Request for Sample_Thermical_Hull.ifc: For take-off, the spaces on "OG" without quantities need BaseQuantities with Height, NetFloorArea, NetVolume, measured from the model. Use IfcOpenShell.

First a look at what the model holds.

```python
import ifcopenshell
import ifcopenshell.util.element
import ifcopenshell.util.unit

model = ifcopenshell.open("Sample_Thermical_Hull.ifc")
print(model.schema)
for unit_type in ("LENGTHUNIT", "AREAUNIT", "VOLUMEUNIT"):
    print(unit_type, ifcopenshell.util.unit.calculate_unit_scale(model, unit_type))
storey = next(s for s in model.by_type("IfcBuildingStorey") if s.Name == "OG")
spaces = [e for e in ifcopenshell.util.element.get_decomposition(storey) if e.is_a("IfcSpace")]
for e in sorted(spaces, key=lambda e: e.id()):
    print(e.id(), e.is_a(), e.Name, list(ifcopenshell.util.element.get_psets(e, qtos_only=True)), sep=" | ")
```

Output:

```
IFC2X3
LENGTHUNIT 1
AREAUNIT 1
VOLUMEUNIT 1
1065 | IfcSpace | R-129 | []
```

```python
import ifcopenshell
import ifcopenshell.api.pset
import ifcopenshell.geom
import ifcopenshell.util.element
import ifcopenshell.util.shape
import ifcopenshell.util.unit

model = ifcopenshell.open("Sample_Thermical_Hull.ifc")
unit_scale = ifcopenshell.util.unit.calculate_unit_scale(model)
area_scale = ifcopenshell.util.unit.calculate_unit_scale(model, "AREAUNIT")
volume_scale = ifcopenshell.util.unit.calculate_unit_scale(model, "VOLUMEUNIT")
settings = ifcopenshell.geom.settings()

storey = next(s for s in model.by_type("IfcBuildingStorey") if s.Name == "OG")
spaces = [e for e in ifcopenshell.util.element.get_decomposition(storey) if e.is_a("IfcSpace")]

for e in sorted(spaces, key=lambda e: e.id()):
    if ifcopenshell.util.element.get_psets(e, qtos_only=True, should_inherit=False):
        continue
    # Geometry comes back in metres, in the element's own axes.
    shape = ifcopenshell.geom.create_shape(settings, e)
    values = {
        "Height": ifcopenshell.util.shape.get_z(shape.geometry) / unit_scale,
        "NetFloorArea": ifcopenshell.util.shape.get_footprint_area(shape.geometry) / area_scale,
        "NetVolume": ifcopenshell.util.shape.get_volume(shape.geometry) / volume_scale,
    }
    qto = ifcopenshell.api.pset.add_qto(model, product=e, name="BaseQuantities")
    ifcopenshell.api.pset.edit_qto(model, qto=qto, properties=values)
    print(e.id(), {k: round(v, 3) for k, v in values.items()})

model.write("Sample_Thermical_Hull_updated.ifc")
```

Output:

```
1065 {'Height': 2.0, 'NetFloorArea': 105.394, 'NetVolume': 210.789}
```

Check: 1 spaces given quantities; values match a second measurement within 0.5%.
